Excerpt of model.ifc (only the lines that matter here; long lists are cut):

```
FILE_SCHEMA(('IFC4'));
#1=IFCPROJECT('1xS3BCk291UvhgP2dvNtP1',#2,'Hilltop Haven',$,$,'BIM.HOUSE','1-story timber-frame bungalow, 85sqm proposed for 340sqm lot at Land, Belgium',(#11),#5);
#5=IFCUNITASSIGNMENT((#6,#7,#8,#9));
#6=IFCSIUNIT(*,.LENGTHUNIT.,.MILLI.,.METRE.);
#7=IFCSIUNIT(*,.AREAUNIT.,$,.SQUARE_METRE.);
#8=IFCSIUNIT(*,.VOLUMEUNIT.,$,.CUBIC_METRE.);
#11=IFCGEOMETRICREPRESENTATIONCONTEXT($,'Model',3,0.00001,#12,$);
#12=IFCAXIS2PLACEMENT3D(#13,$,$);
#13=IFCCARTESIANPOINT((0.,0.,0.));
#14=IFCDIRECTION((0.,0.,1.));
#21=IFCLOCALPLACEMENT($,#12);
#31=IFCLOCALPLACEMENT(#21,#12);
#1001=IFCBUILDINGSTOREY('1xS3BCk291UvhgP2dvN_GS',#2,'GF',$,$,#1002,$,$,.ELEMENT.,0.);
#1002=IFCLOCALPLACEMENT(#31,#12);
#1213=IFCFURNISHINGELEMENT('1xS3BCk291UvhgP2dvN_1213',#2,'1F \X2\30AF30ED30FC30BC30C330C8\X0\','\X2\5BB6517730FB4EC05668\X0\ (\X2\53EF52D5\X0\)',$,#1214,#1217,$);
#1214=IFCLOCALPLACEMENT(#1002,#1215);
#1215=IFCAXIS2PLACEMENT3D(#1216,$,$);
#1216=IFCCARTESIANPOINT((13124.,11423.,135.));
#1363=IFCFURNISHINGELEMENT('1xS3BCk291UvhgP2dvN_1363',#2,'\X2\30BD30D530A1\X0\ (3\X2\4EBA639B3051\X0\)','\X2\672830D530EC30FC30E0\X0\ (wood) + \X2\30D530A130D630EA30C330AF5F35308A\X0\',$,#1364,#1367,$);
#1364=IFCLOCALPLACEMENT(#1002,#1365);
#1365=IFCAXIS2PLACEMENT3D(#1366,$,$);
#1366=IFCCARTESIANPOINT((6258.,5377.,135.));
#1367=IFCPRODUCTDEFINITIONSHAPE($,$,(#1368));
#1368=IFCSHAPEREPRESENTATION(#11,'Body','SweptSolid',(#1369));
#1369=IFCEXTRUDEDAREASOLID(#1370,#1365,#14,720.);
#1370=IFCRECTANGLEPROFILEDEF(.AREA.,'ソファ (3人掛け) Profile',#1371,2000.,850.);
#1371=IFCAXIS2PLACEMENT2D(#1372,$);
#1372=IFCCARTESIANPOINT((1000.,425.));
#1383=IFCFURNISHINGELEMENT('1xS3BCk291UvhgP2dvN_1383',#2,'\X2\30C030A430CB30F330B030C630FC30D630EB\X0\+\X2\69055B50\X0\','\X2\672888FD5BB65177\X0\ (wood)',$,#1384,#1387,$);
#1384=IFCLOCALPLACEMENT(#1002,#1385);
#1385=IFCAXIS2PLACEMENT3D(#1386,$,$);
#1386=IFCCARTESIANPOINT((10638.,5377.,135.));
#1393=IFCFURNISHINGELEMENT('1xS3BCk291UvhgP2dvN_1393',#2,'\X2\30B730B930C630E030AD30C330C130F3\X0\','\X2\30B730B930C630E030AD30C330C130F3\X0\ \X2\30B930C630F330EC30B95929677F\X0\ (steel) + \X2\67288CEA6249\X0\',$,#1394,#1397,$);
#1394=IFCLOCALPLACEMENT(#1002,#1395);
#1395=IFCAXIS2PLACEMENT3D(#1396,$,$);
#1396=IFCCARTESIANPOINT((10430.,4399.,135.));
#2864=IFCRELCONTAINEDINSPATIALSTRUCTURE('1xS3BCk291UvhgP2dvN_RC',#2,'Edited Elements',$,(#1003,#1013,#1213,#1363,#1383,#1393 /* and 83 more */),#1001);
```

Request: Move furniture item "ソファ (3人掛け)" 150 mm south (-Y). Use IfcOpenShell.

```python
import ifcopenshell
import ifcopenshell.api.geometry
import ifcopenshell.util.placement

model = ifcopenshell.open("model.ifc")

item = model.by_guid("1xS3BCk291UvhgP2dvN_1363")
matrix = ifcopenshell.util.placement.get_local_placement(item.ObjectPlacement)
matrix[1, 3] -= 150.0
ifcopenshell.api.geometry.edit_object_placement(model, product=item, matrix=matrix, is_si=False)

print(ifcopenshell.util.placement.get_local_placement(item.ObjectPlacement).round(3) + 0.0)

model.write("model_rev.ifc")
```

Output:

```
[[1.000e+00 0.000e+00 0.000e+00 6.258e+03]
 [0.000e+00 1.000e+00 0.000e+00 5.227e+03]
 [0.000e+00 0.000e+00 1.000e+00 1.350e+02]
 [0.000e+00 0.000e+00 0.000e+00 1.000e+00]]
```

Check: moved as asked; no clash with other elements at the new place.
